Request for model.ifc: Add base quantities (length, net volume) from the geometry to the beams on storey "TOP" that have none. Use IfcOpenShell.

First a look at what the model holds.

```python
import ifcopenshell
import ifcopenshell.util.element
import ifcopenshell.util.unit

model = ifcopenshell.open("model.ifc")
print(model.schema)
for unit_type in ("LENGTHUNIT", "AREAUNIT", "VOLUMEUNIT"):
    print(unit_type, ifcopenshell.util.unit.calculate_unit_scale(model, unit_type))
storey = next(s for s in model.by_type("IfcBuildingStorey") if s.Name == "TOP")
beams = [e for e in ifcopenshell.util.element.get_decomposition(storey) if e.is_a("IfcBeam")]
for e in sorted(beams, key=lambda e: e.id()):
    print(e.id(), e.is_a(), e.Name, list(ifcopenshell.util.element.get_psets(e, qtos_only=True)), sep=" | ")
```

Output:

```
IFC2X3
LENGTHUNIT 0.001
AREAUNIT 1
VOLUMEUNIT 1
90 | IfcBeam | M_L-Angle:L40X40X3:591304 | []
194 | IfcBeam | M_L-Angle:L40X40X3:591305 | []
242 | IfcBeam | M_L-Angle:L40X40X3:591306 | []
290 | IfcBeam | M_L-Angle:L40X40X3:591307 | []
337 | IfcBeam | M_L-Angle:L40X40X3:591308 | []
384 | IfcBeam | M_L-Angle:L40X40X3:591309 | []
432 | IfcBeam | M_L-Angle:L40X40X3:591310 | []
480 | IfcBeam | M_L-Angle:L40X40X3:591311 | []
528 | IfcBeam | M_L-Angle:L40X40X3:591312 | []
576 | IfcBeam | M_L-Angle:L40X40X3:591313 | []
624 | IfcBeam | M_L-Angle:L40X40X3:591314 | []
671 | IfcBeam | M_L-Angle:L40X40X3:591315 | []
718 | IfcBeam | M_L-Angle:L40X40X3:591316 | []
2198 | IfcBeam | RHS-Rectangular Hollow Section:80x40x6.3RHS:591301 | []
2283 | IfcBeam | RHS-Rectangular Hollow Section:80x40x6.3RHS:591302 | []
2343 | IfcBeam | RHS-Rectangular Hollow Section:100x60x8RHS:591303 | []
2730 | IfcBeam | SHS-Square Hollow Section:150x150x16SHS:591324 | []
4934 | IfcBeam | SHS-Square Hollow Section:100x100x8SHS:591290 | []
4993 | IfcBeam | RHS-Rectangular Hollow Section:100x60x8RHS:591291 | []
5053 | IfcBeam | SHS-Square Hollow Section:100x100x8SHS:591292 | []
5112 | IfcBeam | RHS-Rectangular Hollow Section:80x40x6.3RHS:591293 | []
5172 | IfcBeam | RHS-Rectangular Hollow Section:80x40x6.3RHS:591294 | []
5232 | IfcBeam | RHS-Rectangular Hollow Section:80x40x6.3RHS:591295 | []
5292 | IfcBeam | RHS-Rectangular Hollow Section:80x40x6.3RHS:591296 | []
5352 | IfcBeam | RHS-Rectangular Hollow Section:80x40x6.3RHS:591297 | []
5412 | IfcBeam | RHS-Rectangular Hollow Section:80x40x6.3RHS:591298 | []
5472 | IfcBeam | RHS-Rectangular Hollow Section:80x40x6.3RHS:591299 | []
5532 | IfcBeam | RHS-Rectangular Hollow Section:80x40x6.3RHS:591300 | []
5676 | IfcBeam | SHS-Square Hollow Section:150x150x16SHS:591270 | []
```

```python
import ifcopenshell
import ifcopenshell.api.pset
import ifcopenshell.geom
import ifcopenshell.util.element
import ifcopenshell.util.shape
import ifcopenshell.util.unit

model = ifcopenshell.open("model.ifc")
unit_scale = ifcopenshell.util.unit.calculate_unit_scale(model)
volume_scale = ifcopenshell.util.unit.calculate_unit_scale(model, "VOLUMEUNIT")
settings = ifcopenshell.geom.settings()

storey = next(s for s in model.by_type("IfcBuildingStorey") if s.Name == "TOP")
beams = [e for e in ifcopenshell.util.element.get_decomposition(storey) if e.is_a("IfcBeam")]

for e in sorted(beams, key=lambda e: e.id()):
    if ifcopenshell.util.element.get_psets(e, qtos_only=True, should_inherit=False):
        continue
    # Geometry comes back in metres, in the element's own axes.
    shape = ifcopenshell.geom.create_shape(settings, e)
    values = {
        "Length": ifcopenshell.util.shape.get_max_xyz(shape.geometry) / unit_scale,
        "NetVolume": ifcopenshell.util.shape.get_volume(shape.geometry) / volume_scale,
    }
    qto = ifcopenshell.api.pset.add_qto(model, product=e, name="BaseQuantities")
    ifcopenshell.api.pset.edit_qto(model, qto=qto, properties=values)
    print(e.id(), {k: round(v, 3) for k, v in values.items()})

model.write("model_updated.ifc")
```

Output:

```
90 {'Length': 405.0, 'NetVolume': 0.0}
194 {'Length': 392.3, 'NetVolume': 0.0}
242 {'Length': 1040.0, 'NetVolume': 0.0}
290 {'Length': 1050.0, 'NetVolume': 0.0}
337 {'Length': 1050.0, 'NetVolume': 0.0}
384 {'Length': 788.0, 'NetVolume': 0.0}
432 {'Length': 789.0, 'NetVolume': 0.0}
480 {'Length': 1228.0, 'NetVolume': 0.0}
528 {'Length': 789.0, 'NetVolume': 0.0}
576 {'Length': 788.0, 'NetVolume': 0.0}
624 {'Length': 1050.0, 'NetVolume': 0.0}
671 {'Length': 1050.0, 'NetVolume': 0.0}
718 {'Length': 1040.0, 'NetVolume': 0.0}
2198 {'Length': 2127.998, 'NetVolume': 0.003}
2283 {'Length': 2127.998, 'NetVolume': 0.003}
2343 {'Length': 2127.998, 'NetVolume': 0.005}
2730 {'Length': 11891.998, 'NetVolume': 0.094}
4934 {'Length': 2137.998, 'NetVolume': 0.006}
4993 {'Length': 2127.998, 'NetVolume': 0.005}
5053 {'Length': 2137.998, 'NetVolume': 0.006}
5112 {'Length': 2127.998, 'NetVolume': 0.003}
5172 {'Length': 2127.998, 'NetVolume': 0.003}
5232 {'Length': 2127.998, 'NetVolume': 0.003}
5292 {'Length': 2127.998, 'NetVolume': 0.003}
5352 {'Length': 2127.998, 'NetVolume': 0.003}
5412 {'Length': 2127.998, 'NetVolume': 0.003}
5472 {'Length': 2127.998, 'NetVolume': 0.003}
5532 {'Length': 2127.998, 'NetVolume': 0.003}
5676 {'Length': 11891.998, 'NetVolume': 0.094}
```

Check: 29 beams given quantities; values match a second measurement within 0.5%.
